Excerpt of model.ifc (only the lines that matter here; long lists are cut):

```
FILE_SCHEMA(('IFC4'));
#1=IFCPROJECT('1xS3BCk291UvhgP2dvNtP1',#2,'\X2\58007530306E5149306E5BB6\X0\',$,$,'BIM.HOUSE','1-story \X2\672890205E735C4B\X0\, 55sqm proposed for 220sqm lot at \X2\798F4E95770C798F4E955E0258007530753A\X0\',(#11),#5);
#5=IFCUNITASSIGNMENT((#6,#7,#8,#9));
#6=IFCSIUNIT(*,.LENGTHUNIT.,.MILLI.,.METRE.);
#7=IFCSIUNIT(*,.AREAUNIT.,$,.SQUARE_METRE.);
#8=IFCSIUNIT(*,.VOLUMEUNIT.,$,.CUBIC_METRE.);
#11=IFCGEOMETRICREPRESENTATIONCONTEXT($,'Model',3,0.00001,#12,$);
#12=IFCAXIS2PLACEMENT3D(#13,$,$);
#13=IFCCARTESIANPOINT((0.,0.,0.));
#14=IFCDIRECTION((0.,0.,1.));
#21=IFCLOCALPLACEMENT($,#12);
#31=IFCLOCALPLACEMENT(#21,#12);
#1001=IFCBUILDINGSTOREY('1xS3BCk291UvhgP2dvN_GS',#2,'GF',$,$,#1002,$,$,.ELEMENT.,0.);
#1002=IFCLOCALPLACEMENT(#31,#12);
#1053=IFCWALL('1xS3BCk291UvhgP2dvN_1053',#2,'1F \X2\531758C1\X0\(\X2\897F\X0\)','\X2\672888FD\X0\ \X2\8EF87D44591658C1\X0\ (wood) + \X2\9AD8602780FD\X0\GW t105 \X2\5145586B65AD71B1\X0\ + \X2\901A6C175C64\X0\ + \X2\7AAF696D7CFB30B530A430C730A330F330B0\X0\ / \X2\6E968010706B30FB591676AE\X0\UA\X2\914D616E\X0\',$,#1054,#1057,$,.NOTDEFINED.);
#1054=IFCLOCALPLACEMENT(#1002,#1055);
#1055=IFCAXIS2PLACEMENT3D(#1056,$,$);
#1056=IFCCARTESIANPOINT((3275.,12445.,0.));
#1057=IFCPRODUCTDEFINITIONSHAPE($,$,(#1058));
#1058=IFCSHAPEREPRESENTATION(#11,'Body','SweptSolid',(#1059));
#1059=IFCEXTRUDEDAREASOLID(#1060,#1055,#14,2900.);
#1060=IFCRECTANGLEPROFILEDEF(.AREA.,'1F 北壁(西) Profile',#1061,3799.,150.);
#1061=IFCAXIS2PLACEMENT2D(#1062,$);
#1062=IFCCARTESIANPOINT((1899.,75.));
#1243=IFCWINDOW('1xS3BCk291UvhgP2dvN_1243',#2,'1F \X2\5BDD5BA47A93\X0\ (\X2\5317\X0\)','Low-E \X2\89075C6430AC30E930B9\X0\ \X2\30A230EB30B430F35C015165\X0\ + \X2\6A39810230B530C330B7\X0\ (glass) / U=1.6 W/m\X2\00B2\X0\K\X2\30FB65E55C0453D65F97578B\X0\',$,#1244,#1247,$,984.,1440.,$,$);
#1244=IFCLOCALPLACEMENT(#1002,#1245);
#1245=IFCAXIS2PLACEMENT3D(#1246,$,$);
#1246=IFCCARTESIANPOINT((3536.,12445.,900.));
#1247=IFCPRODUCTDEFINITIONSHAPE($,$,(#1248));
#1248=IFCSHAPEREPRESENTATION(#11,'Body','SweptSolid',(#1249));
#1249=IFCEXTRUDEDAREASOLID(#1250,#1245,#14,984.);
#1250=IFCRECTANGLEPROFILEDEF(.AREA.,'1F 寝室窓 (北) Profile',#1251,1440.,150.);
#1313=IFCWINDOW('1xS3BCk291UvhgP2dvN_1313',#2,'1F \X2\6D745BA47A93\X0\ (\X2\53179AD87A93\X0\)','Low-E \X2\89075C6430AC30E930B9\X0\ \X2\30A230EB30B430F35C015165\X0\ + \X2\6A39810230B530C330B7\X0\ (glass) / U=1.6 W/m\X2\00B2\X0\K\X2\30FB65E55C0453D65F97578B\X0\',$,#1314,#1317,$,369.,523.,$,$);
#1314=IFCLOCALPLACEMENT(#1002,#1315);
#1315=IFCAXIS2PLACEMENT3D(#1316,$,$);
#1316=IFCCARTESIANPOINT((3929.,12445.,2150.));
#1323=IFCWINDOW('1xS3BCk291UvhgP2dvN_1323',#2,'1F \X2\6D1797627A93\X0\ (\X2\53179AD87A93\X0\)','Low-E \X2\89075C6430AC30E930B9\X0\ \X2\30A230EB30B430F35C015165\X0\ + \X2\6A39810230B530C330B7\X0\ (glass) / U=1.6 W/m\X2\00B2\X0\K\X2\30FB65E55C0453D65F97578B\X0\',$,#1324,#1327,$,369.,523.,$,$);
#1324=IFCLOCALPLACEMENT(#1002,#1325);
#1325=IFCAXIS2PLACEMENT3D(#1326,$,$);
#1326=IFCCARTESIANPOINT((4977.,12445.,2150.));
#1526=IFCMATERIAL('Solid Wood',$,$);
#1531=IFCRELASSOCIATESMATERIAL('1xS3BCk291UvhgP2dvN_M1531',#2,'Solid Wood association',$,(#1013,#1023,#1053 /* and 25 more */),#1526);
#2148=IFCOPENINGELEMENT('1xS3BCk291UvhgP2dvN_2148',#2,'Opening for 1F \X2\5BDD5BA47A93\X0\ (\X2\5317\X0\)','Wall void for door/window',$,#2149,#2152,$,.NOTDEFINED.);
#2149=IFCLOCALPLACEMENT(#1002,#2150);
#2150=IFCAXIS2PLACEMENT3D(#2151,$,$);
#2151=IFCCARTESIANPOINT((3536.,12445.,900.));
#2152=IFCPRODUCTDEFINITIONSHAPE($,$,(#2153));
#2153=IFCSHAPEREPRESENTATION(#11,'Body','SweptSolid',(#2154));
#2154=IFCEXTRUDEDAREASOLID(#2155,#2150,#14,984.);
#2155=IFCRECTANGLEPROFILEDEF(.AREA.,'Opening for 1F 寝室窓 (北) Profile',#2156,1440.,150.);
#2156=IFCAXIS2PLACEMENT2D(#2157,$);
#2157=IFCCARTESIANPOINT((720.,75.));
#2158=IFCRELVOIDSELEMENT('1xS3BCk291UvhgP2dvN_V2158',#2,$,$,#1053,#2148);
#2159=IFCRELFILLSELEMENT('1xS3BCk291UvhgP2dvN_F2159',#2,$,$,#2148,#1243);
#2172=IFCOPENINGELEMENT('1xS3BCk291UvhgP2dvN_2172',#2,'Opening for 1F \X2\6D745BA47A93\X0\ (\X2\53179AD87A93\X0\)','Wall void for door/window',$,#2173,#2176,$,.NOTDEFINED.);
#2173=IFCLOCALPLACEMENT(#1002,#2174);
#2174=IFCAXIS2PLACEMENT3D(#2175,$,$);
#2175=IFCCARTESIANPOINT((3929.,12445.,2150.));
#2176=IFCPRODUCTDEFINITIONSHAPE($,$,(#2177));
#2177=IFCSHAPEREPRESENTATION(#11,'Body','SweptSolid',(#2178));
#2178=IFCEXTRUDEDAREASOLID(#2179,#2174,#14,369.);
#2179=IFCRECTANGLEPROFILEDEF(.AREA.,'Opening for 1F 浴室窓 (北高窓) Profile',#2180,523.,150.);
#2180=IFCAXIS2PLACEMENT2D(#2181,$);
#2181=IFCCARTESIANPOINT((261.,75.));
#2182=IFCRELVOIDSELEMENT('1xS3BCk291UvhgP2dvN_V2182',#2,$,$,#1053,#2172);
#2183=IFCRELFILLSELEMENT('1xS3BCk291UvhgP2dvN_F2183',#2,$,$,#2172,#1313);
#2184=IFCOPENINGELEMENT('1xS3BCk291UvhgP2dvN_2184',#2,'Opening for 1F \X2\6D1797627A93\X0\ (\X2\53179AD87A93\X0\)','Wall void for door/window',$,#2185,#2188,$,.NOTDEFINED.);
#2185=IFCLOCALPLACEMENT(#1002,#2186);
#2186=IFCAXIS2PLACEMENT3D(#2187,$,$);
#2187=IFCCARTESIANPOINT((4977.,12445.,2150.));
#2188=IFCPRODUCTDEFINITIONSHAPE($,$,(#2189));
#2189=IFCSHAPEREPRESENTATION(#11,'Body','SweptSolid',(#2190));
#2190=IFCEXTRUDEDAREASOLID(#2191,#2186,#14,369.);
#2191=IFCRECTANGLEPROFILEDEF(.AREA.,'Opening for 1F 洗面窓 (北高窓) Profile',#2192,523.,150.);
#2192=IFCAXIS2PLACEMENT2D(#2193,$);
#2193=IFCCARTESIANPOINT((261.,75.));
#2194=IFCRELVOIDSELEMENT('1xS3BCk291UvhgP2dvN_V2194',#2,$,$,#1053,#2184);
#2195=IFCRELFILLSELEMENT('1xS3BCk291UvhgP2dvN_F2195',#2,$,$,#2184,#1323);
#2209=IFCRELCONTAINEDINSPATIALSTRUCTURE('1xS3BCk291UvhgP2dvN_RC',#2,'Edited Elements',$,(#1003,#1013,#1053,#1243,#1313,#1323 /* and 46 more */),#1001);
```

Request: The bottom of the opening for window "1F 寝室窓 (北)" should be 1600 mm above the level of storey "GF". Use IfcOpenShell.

```python
import numpy as np
import ifcopenshell
import ifcopenshell.api.geometry
import ifcopenshell.geom
import ifcopenshell.util.element
import ifcopenshell.util.placement
import ifcopenshell.util.shape
import ifcopenshell.util.unit

model = ifcopenshell.open("model.ifc")
unit_scale = ifcopenshell.util.unit.calculate_unit_scale(model)

window = model.by_id(1243)
opening = window.FillsVoids[0].RelatingOpeningElement
storey = ifcopenshell.util.element.get_container(window, ifc_class="IfcBuildingStorey")
level = ifcopenshell.util.placement.get_local_placement(storey.ObjectPlacement)[2, 3]

# The opening's origin need not be at the sill, so measure its lowest point.
shape = ifcopenshell.geom.create_shape(ifcopenshell.geom.settings(), opening)
bottom = ifcopenshell.util.shape.get_shape_bottom_elevation(shape, shape.geometry) / unit_scale
dz = level + 1.6 / unit_scale - bottom

shift = np.array([0.0, 0.0, dz])
# The window is not placed relative to its opening, so move both.
for product in (opening, window):
    matrix = ifcopenshell.util.placement.get_local_placement(product.ObjectPlacement)
    matrix[:3, 3] += shift
    ifcopenshell.api.geometry.edit_object_placement(model, product=product, matrix=matrix, is_si=False)

print(f"moved by {dz * unit_scale:+.3f} m")

model.write("model_edited.ifc")
```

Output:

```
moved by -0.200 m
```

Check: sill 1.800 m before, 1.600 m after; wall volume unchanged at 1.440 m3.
